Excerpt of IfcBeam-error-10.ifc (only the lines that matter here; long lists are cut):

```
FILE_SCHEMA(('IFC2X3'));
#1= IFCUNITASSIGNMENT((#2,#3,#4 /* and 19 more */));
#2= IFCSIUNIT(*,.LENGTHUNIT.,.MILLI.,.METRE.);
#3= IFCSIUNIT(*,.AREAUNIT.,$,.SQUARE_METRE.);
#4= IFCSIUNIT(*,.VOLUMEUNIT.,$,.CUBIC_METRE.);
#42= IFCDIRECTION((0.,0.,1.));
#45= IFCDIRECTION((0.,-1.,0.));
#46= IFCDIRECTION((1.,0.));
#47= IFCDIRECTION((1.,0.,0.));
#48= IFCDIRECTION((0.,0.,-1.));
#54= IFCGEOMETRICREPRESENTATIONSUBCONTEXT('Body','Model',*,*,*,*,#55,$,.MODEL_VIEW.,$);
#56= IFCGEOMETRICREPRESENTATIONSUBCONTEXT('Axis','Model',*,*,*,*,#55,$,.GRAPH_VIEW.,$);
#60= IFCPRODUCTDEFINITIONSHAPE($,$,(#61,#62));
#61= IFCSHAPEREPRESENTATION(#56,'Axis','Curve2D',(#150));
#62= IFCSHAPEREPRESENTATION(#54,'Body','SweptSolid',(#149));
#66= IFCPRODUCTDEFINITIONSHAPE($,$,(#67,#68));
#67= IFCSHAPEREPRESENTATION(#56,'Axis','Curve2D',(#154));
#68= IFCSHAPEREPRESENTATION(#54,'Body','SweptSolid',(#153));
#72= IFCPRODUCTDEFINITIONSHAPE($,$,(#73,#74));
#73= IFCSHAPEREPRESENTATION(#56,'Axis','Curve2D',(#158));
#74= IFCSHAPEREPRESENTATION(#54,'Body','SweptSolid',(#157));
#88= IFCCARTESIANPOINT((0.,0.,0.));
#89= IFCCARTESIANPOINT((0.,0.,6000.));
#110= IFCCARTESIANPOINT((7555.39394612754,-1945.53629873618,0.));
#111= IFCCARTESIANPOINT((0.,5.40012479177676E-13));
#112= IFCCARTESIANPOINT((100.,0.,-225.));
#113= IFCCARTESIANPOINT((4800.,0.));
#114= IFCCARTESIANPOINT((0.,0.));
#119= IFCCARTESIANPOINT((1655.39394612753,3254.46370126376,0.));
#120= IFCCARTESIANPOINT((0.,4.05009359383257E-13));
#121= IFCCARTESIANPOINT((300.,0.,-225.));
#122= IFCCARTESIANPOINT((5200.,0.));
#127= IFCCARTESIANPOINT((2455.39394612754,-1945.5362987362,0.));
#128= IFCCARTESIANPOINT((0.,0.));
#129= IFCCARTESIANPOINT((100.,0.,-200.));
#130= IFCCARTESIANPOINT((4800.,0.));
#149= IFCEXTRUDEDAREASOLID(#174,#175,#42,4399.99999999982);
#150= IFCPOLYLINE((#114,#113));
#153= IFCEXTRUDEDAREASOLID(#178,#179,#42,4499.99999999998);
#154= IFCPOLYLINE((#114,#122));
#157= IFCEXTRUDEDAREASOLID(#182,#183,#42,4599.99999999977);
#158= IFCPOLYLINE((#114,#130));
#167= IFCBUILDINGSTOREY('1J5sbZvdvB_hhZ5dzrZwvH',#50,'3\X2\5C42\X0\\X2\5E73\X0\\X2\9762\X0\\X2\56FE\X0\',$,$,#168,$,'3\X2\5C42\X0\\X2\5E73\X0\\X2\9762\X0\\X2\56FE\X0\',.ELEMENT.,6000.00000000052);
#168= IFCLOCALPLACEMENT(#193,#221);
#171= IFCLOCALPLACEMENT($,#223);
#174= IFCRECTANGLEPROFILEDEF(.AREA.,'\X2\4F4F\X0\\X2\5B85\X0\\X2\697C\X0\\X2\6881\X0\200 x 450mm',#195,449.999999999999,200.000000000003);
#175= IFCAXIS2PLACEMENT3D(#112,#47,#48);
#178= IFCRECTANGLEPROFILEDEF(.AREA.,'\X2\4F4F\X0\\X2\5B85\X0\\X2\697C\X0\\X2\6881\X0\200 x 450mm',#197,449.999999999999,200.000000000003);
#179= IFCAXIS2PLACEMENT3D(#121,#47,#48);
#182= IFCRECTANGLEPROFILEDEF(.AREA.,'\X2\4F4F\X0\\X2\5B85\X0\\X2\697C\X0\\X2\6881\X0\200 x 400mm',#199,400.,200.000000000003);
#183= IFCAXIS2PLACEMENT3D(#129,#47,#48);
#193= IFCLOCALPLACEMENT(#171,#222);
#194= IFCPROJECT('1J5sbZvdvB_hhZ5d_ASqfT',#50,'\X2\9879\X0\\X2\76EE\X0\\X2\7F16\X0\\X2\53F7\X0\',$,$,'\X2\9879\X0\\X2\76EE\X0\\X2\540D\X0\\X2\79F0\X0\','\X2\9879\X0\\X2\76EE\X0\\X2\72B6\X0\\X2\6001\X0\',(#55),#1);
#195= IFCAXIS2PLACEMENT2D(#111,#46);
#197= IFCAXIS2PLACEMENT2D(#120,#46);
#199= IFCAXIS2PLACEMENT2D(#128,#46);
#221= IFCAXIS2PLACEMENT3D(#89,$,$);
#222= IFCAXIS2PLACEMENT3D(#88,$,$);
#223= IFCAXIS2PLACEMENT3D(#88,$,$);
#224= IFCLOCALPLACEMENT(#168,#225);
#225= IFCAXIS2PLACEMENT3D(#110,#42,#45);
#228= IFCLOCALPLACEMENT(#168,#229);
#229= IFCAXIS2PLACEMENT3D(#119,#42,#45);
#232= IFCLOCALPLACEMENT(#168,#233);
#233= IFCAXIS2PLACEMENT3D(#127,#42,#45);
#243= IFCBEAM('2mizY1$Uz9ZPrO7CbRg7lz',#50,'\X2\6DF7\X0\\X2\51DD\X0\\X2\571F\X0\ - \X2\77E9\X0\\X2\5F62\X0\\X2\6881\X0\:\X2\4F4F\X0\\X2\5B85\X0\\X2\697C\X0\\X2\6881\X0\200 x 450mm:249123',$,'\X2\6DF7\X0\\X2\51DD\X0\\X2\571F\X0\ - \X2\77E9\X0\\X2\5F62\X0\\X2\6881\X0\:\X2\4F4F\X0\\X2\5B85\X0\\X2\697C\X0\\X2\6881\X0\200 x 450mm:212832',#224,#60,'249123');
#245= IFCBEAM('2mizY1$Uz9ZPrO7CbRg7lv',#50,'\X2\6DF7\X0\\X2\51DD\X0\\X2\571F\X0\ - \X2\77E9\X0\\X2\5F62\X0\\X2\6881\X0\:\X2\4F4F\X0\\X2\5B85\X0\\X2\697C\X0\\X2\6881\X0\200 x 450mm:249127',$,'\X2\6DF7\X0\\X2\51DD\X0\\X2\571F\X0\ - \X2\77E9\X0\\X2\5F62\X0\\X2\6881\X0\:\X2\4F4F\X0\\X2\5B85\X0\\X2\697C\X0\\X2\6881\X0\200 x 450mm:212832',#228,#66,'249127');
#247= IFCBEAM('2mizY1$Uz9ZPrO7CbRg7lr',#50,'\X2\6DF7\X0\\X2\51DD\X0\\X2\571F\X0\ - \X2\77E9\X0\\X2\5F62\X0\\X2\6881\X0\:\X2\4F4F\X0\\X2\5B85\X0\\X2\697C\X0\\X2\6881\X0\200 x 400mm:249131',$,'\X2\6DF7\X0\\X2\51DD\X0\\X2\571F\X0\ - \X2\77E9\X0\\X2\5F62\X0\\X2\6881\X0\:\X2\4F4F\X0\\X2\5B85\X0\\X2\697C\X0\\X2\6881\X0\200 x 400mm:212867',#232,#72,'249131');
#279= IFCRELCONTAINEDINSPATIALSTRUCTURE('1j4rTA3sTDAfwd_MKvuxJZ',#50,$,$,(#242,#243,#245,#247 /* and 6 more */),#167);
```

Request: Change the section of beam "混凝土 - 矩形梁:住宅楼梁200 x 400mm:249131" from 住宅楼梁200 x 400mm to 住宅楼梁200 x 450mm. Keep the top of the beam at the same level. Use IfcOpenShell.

```python
import ifcopenshell
import ifcopenshell.util.element
import ifcopenshell.util.representation

model = ifcopenshell.open("IfcBeam-error-10.ifc")

member = model.by_guid("2mizY1$Uz9ZPrO7CbRg7lr")
source = next(p for p in model.by_type("IfcRectangleProfileDef") if p.ProfileName == "住宅楼梁200 x 450mm")

body = ifcopenshell.util.representation.get_representation(member, "Model", "Body")
solid = body.Items[0]
old_profile = solid.SweptArea

# Copy the section's sizes but keep this member's own profile position.
profile = ifcopenshell.util.element.copy(model, source)
# Profiles are centred, so shift by half the change in depth to hold the top.
shift = (old_profile.XDim - profile.XDim) / 2
x, y = old_profile.Position.Location.Coordinates
up = (-1.0, 0.0)  # upwards, in the solid's own plane
location = model.createIfcCartesianPoint((x + up[0] * shift, y + up[1] * shift))
profile.Position = model.createIfcAxis2Placement2D(location, old_profile.Position.RefDirection)
solid.SweptArea = profile
if not model.get_total_inverses(old_profile):
    ifcopenshell.util.element.remove_deep2(model, old_profile)
member.Name = member.Name.replace("住宅楼梁200 x 400mm", "住宅楼梁200 x 450mm")
member.ObjectType = member.ObjectType.replace("住宅楼梁200 x 400mm", "住宅楼梁200 x 450mm")

print(solid.SweptArea)

model.write("IfcBeam-error-10_rev.ifc")
```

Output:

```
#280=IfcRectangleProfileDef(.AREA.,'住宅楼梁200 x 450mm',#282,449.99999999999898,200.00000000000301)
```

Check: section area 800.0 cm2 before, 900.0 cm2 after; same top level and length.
